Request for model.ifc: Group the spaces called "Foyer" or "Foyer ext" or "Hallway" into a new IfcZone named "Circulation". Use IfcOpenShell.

First a look at what the model holds.

```python
import ifcopenshell

model = ifcopenshell.open("model.ifc")
print(model.schema)
seen = {}
for space in model.by_type("IfcSpace"):
    seen[space.LongName] = seen.get(space.LongName, 0) + 1
for name, count in sorted(seen.items(), key=str):
    print(count, "x", name)
print("zones:", [z.Name for z in model.by_type("IfcZone")][:20])
```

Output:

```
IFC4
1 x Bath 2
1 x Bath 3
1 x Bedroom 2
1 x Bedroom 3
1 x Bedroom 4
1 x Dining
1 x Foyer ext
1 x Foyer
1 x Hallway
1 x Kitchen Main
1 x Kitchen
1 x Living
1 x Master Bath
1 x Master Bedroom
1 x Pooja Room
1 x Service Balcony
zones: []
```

```python
import ifcopenshell
import ifcopenshell.api.group
import ifcopenshell.api.root

model = ifcopenshell.open("model.ifc")

names = {"Foyer", "Foyer ext", "Hallway"}
spaces = [s for s in model.by_type("IfcSpace") if s.LongName in names]

zone = ifcopenshell.api.root.create_entity(model, ifc_class="IfcZone", name="Circulation")
ifcopenshell.api.group.assign_group(model, products=spaces, group=zone)
print(len(spaces), "spaces in", zone.Name)

model.write("model_v2.ifc")
```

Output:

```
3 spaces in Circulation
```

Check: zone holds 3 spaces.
